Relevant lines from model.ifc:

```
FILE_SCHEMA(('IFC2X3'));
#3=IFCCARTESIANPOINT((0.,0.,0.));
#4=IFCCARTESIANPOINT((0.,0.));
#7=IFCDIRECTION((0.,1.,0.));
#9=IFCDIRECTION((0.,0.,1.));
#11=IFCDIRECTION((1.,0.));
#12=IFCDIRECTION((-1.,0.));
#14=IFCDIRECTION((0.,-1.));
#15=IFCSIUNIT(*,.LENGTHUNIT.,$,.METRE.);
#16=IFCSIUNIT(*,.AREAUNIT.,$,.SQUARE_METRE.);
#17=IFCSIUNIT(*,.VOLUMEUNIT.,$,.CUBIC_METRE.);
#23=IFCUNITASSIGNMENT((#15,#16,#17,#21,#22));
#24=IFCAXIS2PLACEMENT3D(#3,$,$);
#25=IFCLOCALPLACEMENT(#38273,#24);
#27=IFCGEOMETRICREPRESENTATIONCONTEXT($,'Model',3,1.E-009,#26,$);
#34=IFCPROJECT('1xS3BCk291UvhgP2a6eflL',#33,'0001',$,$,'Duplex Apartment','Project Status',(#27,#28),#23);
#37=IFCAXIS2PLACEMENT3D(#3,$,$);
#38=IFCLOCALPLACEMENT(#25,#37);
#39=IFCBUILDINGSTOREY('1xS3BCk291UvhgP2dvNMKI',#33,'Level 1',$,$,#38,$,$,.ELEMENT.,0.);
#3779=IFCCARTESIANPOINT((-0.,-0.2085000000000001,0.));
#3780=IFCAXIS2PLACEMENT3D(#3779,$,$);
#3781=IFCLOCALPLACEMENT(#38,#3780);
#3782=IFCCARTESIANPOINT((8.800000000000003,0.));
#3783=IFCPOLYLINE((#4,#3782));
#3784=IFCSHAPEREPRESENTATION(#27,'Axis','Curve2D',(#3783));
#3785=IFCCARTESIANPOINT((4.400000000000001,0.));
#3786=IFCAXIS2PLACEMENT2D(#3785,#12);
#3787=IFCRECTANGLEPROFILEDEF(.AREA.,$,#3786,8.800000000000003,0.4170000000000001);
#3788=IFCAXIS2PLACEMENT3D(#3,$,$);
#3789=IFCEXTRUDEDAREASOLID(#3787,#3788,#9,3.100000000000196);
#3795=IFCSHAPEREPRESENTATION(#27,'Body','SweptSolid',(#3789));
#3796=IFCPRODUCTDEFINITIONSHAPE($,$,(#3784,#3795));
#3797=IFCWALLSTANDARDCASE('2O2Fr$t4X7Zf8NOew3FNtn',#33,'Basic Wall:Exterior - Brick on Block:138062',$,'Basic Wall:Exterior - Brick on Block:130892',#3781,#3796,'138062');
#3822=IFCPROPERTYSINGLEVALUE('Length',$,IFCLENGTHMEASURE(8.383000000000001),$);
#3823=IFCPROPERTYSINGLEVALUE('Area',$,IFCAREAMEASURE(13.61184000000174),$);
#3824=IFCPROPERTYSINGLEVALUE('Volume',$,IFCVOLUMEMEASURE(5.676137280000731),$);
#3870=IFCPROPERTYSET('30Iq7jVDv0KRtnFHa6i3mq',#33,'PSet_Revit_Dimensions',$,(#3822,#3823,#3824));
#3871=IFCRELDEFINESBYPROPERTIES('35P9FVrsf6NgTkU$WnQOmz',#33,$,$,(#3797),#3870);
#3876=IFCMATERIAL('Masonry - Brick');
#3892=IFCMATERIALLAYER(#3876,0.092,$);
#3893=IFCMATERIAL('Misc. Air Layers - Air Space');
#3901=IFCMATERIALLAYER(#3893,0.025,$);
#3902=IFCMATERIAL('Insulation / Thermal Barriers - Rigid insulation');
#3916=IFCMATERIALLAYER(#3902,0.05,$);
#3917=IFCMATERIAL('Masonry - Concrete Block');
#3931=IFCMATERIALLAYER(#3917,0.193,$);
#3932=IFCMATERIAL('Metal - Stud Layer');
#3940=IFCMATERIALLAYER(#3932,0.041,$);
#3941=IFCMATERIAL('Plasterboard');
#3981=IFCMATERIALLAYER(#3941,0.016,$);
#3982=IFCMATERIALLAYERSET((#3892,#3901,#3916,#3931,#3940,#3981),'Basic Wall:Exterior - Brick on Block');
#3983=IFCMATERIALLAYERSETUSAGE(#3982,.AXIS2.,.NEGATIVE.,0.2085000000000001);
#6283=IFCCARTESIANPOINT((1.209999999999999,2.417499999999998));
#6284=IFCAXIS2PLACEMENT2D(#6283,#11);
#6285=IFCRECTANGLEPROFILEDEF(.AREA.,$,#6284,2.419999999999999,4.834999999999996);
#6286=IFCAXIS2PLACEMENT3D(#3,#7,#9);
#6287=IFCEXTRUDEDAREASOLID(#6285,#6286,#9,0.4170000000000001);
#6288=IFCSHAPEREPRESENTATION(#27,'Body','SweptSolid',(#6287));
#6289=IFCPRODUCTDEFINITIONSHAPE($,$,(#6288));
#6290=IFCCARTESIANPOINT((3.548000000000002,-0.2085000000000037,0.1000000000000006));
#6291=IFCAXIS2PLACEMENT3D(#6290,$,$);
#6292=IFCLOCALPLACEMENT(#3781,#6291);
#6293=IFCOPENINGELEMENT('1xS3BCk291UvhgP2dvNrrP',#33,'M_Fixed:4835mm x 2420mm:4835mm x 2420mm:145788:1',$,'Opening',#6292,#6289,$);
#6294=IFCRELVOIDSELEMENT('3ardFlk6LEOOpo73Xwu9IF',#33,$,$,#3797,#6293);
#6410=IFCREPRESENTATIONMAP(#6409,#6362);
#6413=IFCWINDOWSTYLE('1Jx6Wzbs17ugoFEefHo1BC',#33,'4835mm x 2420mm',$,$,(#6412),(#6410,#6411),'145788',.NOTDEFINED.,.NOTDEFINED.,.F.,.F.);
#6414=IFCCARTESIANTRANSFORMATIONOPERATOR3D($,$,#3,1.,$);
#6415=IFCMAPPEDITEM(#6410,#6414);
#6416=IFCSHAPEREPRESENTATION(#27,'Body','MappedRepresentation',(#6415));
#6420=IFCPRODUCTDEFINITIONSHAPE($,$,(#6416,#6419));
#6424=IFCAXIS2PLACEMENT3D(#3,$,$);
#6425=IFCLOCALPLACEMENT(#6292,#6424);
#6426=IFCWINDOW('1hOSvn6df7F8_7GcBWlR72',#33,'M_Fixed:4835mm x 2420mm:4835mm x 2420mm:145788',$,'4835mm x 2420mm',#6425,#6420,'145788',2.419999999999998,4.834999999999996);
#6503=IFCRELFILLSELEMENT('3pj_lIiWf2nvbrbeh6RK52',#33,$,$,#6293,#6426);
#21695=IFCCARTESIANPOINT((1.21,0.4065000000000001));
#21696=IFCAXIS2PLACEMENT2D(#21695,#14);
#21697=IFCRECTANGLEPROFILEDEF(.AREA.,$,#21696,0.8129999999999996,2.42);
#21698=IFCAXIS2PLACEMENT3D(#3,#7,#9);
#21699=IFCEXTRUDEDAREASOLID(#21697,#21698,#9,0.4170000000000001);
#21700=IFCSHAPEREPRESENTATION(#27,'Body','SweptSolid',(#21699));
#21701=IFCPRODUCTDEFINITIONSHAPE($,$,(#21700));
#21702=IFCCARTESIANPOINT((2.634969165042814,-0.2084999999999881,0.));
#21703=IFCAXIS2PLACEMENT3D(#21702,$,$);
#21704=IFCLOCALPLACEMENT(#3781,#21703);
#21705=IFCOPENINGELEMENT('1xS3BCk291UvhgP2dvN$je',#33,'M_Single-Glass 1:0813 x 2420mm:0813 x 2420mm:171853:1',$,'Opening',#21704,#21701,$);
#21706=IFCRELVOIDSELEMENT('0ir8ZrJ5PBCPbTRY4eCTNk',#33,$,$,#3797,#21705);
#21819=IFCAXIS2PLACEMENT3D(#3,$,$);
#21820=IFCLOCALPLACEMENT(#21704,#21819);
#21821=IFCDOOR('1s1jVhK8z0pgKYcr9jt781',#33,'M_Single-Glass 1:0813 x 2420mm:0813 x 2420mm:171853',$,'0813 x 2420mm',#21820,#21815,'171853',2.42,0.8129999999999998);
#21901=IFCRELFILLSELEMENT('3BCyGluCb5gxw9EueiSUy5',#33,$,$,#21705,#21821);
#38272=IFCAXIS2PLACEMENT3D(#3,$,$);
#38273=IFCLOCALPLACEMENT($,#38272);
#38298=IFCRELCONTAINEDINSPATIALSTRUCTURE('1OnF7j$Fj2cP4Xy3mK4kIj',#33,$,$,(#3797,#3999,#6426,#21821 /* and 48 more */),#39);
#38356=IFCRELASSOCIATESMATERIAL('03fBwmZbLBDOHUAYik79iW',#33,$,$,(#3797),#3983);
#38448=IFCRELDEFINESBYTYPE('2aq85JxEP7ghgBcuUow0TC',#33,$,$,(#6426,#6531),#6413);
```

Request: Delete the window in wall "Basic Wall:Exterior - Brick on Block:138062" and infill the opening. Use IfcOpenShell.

```python
import ifcopenshell
import ifcopenshell.api.feature
import ifcopenshell.api.pset
import ifcopenshell.api.root
import ifcopenshell.geom
import ifcopenshell.util.element
import ifcopenshell.util.shape
import ifcopenshell.util.unit

model = ifcopenshell.open("model.ifc")
area_scale = ifcopenshell.util.unit.calculate_unit_scale(model, "AREAUNIT")
volume_scale = ifcopenshell.util.unit.calculate_unit_scale(model, "VOLUMEUNIT")
settings = ifcopenshell.geom.settings()


def volume(element):
    """Net volume in cubic metres, openings subtracted."""
    shape = ifcopenshell.geom.create_shape(settings, element)
    return ifcopenshell.util.shape.get_volume(shape.geometry)


window = model.by_guid("1hOSvn6df7F8_7GcBWlR72")
opening = window.FillsVoids[0].RelatingOpeningElement
wall = opening.VoidsElements[0].RelatingBuildingElement
before = volume(wall)

ifcopenshell.api.root.remove_product(model, product=window)
ifcopenshell.api.feature.remove_feature(model, feature=opening)

after = volume(wall)
thickness = 0.417  # wall thickness in metres

# Update the wall's stored quantities.
pset = model.by_id(ifcopenshell.util.element.get_pset(wall, "PSet_Revit_Dimensions", should_inherit=False)["id"])
ifcopenshell.api.pset.edit_pset(model, pset=pset, properties={
    "Area": model.create_entity("IfcAreaMeasure", after / thickness / area_scale),
    "Volume": model.create_entity("IfcVolumeMeasure", after / volume_scale),
})

print(f"wall volume {before:.3f} -> {after:.3f} m3")

model.write("model_updated.ifc")
```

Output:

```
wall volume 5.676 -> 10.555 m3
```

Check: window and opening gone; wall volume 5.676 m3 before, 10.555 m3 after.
